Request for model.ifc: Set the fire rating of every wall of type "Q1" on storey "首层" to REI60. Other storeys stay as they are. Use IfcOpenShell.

First a look at what the model holds.

```python
import ifcopenshell
import ifcopenshell.util.element

model = ifcopenshell.open("model.ifc")
print(model.schema)
storey = next(s for s in model.by_type("IfcBuildingStorey") if s.Name == "首层")
walls = [e for e in ifcopenshell.util.element.get_decomposition(storey) if e.is_a("IfcWall")]
seen = {}
for e in walls:
    element_type = ifcopenshell.util.element.get_type(e)
    key = (element_type.Name if element_type != e and element_type else None, ifcopenshell.util.element.get_pset(e, "Pset_WallCommon", "FireRating"))
    seen[key] = seen.get(key, 0) + 1
for (name, value), count in sorted(seen.items(), key=str):
    print(count, "x", name, "|", value)
```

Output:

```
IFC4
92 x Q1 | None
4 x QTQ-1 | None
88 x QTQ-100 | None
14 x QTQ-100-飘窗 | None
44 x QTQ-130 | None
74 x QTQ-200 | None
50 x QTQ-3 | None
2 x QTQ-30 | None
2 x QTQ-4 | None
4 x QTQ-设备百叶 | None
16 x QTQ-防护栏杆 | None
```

```python
import ifcopenshell
import ifcopenshell.api.pset
import ifcopenshell.util.element

model = ifcopenshell.open("model.ifc")

storey = next(s for s in model.by_type("IfcBuildingStorey") if s.Name == "首层")
walls = [e for e in ifcopenshell.util.element.get_decomposition(storey) if e.is_a("IfcWall")]

count = 0
for e in walls:
    element_type = ifcopenshell.util.element.get_type(e)
    if element_type in (None, e) or element_type.Name != "Q1":
        continue
    # add_pset returns the element's existing set when there is one.
    pset = ifcopenshell.api.pset.add_pset(model, product=e, name="Pset_WallCommon")
    ifcopenshell.api.pset.edit_pset(model, pset=pset, properties={"FireRating": "REI60"})
    count += 1

print(count, "walls updated")

model.write("model-out.ifc")
```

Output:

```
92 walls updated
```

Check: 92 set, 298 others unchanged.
